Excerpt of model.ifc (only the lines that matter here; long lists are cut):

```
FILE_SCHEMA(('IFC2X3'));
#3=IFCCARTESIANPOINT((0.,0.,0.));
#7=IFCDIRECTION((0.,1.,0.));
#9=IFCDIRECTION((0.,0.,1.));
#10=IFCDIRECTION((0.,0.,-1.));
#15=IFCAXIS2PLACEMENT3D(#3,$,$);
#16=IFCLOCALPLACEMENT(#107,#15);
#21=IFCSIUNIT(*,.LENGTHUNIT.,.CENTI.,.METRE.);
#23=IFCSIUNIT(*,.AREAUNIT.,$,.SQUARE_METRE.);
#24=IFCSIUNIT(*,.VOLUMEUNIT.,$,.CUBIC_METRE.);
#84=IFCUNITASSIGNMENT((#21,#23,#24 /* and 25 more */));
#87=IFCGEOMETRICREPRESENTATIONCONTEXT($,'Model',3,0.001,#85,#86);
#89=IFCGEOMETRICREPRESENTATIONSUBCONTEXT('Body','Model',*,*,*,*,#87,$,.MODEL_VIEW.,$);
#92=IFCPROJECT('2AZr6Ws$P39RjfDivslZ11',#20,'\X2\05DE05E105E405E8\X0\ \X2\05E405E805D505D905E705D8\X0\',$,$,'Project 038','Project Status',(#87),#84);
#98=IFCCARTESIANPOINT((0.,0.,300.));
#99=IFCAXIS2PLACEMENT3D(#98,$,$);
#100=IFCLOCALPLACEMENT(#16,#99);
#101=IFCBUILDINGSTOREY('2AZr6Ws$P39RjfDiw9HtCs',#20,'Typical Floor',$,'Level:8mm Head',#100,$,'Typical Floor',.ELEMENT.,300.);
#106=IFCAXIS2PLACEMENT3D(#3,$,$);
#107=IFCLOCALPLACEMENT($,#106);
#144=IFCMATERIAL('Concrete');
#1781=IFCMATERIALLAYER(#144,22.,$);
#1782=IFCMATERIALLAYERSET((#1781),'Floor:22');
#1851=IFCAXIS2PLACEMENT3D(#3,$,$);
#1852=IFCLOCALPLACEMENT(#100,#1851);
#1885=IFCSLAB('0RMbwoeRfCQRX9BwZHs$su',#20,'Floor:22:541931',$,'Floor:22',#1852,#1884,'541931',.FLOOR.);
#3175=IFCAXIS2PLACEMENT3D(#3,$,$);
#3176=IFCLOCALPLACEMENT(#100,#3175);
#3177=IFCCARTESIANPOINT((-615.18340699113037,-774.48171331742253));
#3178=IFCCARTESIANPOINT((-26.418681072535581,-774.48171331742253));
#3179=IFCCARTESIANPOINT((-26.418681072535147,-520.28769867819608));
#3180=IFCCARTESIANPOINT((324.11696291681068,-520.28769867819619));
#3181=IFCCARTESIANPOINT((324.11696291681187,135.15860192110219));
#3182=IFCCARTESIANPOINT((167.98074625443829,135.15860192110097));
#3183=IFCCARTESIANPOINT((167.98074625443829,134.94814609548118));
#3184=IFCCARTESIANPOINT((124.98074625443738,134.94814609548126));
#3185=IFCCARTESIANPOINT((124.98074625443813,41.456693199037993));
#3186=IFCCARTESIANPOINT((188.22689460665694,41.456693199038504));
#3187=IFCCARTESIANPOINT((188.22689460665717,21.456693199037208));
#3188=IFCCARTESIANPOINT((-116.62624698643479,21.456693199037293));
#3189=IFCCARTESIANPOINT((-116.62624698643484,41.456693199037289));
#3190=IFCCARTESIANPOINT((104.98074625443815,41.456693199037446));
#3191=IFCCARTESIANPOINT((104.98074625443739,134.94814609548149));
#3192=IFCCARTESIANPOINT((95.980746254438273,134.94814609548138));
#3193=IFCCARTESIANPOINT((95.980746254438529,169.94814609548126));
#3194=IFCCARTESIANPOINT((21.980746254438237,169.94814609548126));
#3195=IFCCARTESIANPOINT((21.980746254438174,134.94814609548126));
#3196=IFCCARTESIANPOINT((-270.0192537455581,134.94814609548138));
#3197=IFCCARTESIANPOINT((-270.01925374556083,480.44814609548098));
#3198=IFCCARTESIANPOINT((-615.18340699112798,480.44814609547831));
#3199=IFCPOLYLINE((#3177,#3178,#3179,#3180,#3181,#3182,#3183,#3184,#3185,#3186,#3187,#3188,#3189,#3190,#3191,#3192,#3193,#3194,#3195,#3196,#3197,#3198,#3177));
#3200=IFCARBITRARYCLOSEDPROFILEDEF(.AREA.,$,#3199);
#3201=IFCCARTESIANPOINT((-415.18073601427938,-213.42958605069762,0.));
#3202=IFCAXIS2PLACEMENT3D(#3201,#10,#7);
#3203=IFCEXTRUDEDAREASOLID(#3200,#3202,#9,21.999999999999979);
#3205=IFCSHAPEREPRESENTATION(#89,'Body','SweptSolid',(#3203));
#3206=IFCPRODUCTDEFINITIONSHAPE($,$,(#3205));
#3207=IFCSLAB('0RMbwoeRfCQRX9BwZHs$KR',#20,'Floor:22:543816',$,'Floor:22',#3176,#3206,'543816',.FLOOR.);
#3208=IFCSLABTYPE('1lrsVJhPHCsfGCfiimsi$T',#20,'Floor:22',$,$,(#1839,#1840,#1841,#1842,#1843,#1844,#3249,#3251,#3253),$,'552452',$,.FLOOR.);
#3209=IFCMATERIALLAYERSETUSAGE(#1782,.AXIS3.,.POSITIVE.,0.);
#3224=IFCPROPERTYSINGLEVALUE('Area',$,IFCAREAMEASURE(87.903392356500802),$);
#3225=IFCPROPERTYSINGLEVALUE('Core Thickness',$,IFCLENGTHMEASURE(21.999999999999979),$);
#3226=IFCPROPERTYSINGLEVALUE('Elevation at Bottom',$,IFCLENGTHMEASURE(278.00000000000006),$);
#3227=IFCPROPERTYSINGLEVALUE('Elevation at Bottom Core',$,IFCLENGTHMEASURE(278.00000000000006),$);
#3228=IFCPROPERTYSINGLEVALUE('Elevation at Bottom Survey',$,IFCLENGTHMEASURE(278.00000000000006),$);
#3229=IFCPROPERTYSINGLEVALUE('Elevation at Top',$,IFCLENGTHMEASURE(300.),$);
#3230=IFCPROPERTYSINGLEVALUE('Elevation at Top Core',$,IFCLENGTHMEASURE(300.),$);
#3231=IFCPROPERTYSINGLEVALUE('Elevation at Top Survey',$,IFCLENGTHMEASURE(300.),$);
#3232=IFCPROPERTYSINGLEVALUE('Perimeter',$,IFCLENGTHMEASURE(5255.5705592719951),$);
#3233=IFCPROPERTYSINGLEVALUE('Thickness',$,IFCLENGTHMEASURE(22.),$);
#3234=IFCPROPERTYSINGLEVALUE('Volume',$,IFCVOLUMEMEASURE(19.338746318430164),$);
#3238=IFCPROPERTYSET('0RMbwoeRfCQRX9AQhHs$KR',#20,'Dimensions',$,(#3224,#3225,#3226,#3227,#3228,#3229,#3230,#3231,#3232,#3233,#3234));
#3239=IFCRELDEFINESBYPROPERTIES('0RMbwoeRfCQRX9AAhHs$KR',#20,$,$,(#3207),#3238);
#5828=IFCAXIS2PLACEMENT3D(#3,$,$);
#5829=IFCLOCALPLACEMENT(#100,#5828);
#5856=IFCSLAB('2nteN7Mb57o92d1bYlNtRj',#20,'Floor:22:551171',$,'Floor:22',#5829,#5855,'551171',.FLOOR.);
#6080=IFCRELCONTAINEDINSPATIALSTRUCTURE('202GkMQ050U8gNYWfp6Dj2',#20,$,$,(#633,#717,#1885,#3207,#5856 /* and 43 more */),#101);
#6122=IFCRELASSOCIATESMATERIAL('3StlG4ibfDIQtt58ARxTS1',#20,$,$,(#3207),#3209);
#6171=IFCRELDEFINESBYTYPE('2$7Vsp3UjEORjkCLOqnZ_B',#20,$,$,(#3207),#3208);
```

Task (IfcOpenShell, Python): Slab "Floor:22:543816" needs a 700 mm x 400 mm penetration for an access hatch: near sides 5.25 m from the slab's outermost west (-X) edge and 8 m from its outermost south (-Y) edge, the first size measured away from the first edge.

```python
import numpy as np
import ifcopenshell
import ifcopenshell.api.feature
import ifcopenshell.api.geometry
import ifcopenshell.api.pset
import ifcopenshell.api.root
import ifcopenshell.geom
import ifcopenshell.util.element
import ifcopenshell.util.placement
import ifcopenshell.util.representation
import ifcopenshell.util.shape
import ifcopenshell.util.unit

model = ifcopenshell.open("model.ifc")
unit_scale = ifcopenshell.util.unit.calculate_unit_scale(model)
area_scale = ifcopenshell.util.unit.calculate_unit_scale(model, "AREAUNIT")
volume_scale = ifcopenshell.util.unit.calculate_unit_scale(model, "VOLUMEUNIT")
settings = ifcopenshell.geom.settings()


def volume(element):
    """Net volume in cubic metres, openings subtracted."""
    shape = ifcopenshell.geom.create_shape(settings, element)
    return ifcopenshell.util.shape.get_volume(shape.geometry)


slab = model.by_guid("0RMbwoeRfCQRX9BwZHs$KR")
before = volume(slab)

# Extent in the slab's own axes, in metres. The edges named are its -X and -Y sides.
slab_shape = ifcopenshell.geom.create_shape(settings, slab)
vertices = ifcopenshell.util.shape.get_vertices(slab_shape.geometry)
x_min, y_min, bottom = vertices.min(axis=0)
top = vertices[:, 2].max()

opening = ifcopenshell.api.root.create_entity(model, ifc_class="IfcOpeningElement", name="Access hatch opening")
context = ifcopenshell.util.representation.get_context(model, "Model", "Body", "MODEL_VIEW")
width, depth = 0.7, 0.4
outline = [(0.0, 0.0), (width, 0.0), (width, depth), (0.0, depth), (0.0, 0.0)]
# Overshoot both faces by 50 mm so the cut is clean.
shape = ifcopenshell.api.geometry.add_slab_representation(
    model, context=context, depth=top - bottom + 0.1, polyline=outline
)
ifcopenshell.api.geometry.assign_representation(model, product=opening, representation=shape)

matrix = ifcopenshell.util.placement.get_local_placement(slab.ObjectPlacement)
matrix[:, 3] = matrix @ np.append(np.array([x_min + 5.25, y_min + 8, bottom - 0.05]) / unit_scale, 1.0)
ifcopenshell.api.geometry.edit_object_placement(model, product=opening, matrix=matrix, is_si=False)
ifcopenshell.api.feature.add_feature(model, feature=opening, element=slab)

after = volume(slab)

# Update the slab's stored quantities.
pset = model.by_id(ifcopenshell.util.element.get_pset(slab, "Dimensions", should_inherit=False)["id"])
ifcopenshell.api.pset.edit_pset(model, pset=pset, properties={
    "Area": model.create_entity("IfcAreaMeasure", after / (top - bottom) / area_scale),
    "Volume": model.create_entity("IfcVolumeMeasure", after / volume_scale),
})

print(f"slab volume {before:.3f} -> {after:.3f} m3")

model.write("model_rev.ifc")
```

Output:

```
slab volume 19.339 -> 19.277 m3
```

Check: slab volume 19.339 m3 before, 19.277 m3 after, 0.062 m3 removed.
